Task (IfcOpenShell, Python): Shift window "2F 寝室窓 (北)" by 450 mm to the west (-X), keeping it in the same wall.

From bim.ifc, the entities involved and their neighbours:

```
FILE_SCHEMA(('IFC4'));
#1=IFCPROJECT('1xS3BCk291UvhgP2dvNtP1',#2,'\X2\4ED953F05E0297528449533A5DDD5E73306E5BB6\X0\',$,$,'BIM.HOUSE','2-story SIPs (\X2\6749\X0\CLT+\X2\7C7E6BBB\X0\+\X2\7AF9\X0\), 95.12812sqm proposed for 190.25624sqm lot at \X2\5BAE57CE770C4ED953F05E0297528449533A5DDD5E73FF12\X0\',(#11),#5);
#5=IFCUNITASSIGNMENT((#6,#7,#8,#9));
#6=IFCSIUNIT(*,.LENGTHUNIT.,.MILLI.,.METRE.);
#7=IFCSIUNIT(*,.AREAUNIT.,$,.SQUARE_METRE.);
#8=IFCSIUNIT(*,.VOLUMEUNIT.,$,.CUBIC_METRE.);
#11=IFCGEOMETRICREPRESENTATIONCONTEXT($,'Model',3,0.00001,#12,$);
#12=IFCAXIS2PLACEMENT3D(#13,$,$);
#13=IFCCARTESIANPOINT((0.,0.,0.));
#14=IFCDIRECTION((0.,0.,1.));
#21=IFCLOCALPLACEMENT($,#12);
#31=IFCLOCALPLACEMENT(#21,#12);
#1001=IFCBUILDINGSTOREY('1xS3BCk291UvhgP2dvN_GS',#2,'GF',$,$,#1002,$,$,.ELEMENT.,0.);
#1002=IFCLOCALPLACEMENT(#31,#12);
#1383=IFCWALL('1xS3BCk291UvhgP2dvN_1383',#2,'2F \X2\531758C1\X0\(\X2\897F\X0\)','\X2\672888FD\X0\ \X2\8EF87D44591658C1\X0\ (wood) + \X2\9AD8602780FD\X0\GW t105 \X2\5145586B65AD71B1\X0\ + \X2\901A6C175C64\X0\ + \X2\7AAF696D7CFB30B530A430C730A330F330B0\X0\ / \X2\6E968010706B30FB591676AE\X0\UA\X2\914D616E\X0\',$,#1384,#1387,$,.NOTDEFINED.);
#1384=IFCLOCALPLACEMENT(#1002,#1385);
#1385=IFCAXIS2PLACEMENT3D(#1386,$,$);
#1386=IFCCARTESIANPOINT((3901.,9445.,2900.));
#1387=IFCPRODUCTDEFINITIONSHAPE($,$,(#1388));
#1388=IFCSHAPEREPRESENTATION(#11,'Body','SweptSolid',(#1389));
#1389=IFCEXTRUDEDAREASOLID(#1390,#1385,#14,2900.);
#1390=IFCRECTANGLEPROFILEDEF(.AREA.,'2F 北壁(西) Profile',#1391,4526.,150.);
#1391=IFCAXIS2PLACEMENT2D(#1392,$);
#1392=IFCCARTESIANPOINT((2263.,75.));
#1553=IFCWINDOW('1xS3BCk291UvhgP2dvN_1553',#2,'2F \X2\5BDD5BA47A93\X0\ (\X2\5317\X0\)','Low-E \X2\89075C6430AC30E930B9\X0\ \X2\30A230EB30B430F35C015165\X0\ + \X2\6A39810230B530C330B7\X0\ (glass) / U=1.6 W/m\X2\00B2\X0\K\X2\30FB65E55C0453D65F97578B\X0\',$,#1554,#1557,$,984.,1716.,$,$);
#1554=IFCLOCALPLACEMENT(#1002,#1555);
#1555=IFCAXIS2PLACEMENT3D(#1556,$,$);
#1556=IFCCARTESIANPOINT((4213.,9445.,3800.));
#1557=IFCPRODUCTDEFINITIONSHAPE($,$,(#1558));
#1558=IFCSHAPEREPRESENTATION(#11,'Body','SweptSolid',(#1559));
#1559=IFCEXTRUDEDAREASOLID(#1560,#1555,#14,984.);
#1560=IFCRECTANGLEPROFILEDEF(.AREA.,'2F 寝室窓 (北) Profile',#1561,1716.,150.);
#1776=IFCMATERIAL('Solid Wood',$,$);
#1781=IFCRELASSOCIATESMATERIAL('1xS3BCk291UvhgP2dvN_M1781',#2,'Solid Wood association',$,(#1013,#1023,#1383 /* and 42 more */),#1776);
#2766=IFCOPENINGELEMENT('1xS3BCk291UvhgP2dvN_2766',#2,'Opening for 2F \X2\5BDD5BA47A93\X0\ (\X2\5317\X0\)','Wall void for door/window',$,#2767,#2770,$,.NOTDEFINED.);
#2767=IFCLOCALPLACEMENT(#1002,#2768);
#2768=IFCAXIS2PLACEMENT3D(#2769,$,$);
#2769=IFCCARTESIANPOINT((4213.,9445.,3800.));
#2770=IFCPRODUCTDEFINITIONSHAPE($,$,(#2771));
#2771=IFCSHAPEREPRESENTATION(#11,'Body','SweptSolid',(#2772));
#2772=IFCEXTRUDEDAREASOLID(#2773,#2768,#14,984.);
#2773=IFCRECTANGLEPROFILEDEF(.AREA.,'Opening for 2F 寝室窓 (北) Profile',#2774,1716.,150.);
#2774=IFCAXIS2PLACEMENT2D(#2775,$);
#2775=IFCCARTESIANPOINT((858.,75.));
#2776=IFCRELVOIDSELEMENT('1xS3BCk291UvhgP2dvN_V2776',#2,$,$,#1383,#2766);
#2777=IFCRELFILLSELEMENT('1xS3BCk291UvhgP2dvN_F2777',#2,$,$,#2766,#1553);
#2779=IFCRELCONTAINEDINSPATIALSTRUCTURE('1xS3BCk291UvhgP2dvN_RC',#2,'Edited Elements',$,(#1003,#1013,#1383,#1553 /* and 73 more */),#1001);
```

```python
import ifcopenshell
import ifcopenshell.api.geometry
import ifcopenshell.util.placement

model = ifcopenshell.open("bim.ifc")

window = model.by_guid("1xS3BCk291UvhgP2dvN_1553")
opening = window.FillsVoids[0].RelatingOpeningElement
wall = opening.VoidsElements[0].RelatingBuildingElement

wall_matrix = ifcopenshell.util.placement.get_local_placement(wall.ObjectPlacement)
shift = wall_matrix[:3, 0] * -450.0
before = ifcopenshell.util.placement.get_local_placement(window.ObjectPlacement)[:3, 3].copy()

# The window is not placed relative to its opening, so move both.
for product in (opening, window):
    matrix = ifcopenshell.util.placement.get_local_placement(product.ObjectPlacement)
    matrix[:3, 3] += shift
    ifcopenshell.api.geometry.edit_object_placement(model, product=product, matrix=matrix, is_si=False)

after = ifcopenshell.util.placement.get_local_placement(window.ObjectPlacement)[:3, 3]
print("window moved by", (after - before).round(3) + 0.0)

model.write("bim_v2.ifc")
```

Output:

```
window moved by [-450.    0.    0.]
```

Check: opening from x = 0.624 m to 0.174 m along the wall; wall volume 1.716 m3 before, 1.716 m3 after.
